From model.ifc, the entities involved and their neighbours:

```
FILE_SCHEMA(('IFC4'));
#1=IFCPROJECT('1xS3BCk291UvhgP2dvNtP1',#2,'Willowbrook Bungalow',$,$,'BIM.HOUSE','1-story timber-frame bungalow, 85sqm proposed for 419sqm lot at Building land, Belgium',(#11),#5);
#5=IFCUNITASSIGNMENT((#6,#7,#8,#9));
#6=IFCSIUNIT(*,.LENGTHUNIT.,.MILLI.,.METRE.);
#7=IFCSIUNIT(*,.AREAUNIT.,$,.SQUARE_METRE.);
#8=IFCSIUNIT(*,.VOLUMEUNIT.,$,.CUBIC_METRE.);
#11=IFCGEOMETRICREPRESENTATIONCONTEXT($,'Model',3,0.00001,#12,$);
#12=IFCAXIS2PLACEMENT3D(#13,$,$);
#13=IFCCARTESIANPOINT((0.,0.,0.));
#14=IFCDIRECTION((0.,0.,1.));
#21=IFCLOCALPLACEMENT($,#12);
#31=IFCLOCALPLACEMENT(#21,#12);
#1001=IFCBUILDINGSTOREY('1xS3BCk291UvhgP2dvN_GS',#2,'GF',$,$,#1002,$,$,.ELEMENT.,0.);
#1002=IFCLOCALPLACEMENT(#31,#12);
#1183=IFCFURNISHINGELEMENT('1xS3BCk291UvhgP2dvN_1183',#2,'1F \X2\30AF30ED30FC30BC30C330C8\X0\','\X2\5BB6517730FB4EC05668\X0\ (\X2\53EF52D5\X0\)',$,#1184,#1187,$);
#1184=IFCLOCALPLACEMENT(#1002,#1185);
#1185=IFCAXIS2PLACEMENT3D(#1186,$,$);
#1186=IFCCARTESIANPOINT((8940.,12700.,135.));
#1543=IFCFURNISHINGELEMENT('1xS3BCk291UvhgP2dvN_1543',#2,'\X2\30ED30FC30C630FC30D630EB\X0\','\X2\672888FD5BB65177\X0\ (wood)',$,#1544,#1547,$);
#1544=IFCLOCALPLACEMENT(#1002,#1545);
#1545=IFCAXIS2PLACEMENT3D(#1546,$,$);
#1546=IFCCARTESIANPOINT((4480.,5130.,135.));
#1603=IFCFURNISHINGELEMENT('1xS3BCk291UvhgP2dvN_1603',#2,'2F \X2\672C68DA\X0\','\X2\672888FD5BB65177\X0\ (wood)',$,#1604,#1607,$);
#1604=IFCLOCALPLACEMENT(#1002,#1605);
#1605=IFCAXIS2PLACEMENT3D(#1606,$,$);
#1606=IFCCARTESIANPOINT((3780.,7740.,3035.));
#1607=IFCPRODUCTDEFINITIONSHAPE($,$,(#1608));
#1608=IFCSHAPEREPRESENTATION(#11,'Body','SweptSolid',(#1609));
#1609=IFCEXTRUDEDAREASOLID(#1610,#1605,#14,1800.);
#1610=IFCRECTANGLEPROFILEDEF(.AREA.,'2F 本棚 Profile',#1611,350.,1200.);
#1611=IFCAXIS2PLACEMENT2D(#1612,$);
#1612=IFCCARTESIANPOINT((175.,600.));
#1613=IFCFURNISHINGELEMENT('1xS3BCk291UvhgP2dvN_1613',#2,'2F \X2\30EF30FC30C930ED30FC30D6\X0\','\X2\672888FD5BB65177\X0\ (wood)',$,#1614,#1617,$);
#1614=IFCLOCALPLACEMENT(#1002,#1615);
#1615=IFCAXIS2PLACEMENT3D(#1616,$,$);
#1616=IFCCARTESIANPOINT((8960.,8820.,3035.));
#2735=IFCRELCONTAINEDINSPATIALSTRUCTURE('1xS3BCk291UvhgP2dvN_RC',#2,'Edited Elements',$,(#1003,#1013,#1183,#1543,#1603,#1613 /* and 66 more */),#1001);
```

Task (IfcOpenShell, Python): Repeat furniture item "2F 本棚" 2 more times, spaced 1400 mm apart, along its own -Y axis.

```python
import ifcopenshell
import ifcopenshell.api.geometry
import ifcopenshell.api.root
import ifcopenshell.util.element
import ifcopenshell.util.placement
import ifcopenshell.util.unit

model = ifcopenshell.open("model.ifc")
unit_scale = ifcopenshell.util.unit.calculate_unit_scale(model)


def reuse_history(source, copy):
    """copy_class also copies each property set's owner history, people and application; keep the originals."""
    for rel in copy.IsDefinedBy:
        if rel.is_a("IfcRelDefinesByProperties") and (history := rel.RelatingPropertyDefinition.OwnerHistory):
            rel.RelatingPropertyDefinition.OwnerHistory = source.OwnerHistory
            ifcopenshell.util.element.remove_deep2(model, history)


source = model.by_id(1603)
base = ifcopenshell.util.placement.get_local_placement(source.ObjectPlacement)
step = -base[:3, 1] * 1.4 / unit_scale

for i in range(1, 3):
    copy = ifcopenshell.api.root.copy_class(model, product=source)
    copy.Representation = ifcopenshell.util.element.copy_deep(
        model, source.Representation, exclude=["IfcGeometricRepresentationContext", "IfcRepresentationMap"]
    )
    reuse_history(source, copy)
    matrix = base.copy()
    matrix[:3, 3] += i * step
    print("added at", matrix[:3, 3].round(3) + 0.0)
    ifcopenshell.api.geometry.edit_object_placement(model, product=copy, matrix=matrix, is_si=False)

model.write("model_updated.ifc")
```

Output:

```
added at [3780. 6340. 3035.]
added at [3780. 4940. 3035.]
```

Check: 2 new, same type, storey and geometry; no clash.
